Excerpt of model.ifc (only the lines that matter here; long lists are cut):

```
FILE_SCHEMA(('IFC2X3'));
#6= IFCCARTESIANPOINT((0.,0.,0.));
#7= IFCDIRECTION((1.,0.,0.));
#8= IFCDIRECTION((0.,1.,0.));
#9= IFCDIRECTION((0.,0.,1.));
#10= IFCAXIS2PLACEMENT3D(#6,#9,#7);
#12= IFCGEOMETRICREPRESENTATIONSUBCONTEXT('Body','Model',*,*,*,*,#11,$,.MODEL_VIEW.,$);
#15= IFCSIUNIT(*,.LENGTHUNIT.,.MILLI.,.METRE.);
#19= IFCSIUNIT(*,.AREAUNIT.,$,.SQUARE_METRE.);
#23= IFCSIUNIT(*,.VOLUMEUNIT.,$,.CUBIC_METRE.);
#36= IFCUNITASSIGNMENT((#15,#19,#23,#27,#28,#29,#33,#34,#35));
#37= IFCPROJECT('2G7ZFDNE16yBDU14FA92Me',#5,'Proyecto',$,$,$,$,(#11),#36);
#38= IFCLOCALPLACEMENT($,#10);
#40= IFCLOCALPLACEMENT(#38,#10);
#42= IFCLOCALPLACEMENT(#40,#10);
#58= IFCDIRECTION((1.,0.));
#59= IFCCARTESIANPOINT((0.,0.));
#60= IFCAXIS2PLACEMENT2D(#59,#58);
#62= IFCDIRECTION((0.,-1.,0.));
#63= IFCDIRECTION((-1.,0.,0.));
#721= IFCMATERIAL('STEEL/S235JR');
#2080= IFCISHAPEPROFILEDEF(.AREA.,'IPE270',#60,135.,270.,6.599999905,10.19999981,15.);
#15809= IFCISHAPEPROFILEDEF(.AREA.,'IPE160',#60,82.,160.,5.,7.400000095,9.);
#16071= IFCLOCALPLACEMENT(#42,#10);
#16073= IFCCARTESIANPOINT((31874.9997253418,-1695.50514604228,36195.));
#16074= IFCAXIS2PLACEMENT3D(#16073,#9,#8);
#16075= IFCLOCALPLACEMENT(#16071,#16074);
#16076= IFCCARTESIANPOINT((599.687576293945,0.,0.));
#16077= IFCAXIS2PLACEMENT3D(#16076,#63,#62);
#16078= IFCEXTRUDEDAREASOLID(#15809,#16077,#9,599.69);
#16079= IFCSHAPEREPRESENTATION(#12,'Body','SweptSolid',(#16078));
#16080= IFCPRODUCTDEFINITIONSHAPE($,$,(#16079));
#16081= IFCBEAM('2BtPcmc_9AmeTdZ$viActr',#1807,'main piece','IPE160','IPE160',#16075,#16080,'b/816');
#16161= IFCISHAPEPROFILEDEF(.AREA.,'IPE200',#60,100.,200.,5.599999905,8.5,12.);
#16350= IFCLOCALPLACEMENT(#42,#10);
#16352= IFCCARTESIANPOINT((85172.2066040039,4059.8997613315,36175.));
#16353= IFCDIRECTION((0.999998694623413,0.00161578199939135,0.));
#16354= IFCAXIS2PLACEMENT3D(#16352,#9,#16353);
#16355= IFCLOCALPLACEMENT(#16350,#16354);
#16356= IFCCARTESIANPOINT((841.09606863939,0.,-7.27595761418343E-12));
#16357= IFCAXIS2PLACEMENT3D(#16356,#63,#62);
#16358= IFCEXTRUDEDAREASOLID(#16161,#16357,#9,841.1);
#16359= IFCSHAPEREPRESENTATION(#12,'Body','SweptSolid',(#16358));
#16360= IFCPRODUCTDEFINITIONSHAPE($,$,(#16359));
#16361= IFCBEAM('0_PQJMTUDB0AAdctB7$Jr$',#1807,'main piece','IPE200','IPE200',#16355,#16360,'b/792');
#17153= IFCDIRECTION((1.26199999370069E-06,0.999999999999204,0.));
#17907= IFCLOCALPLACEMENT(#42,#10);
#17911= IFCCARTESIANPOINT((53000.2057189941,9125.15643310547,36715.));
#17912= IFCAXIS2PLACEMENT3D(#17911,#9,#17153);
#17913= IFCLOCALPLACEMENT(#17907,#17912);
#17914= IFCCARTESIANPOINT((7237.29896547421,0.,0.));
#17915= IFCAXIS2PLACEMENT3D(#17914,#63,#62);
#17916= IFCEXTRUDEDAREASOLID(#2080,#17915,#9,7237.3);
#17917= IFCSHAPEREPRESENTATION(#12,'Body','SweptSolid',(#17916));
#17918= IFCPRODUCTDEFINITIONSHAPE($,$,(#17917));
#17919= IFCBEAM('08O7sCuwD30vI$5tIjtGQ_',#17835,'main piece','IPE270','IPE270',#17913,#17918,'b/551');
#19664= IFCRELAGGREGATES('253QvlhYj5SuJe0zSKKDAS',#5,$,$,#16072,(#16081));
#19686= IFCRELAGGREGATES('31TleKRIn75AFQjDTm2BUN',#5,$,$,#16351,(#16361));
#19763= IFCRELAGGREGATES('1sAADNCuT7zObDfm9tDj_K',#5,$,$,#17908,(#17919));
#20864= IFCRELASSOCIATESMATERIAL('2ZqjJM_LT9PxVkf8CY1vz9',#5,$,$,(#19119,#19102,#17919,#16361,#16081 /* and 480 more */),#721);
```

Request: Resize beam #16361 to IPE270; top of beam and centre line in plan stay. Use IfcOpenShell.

```python
import ifcopenshell
import ifcopenshell.util.element
import ifcopenshell.util.representation

model = ifcopenshell.open("model.ifc")

member = model.by_guid("0_PQJMTUDB0AAdctB7$Jr$")
source = next(p for p in model.by_type("IfcIShapeProfileDef") if p.ProfileName == "IPE270")

body = ifcopenshell.util.representation.get_representation(member, "Model", "Body")
solid = body.Items[0]
old_profile = solid.SweptArea

# Copy the section's sizes but keep this member's own profile position.
profile = ifcopenshell.util.element.copy(model, source)
# Profiles are centred, so shift by half the change in depth to hold the top.
shift = (old_profile.OverallDepth - profile.OverallDepth) / 2
x, y = old_profile.Position.Location.Coordinates
up = (0.0, 1.0)  # upwards, in the solid's own plane
location = model.createIfcCartesianPoint((x + up[0] * shift, y + up[1] * shift))
profile.Position = model.createIfcAxis2Placement2D(location, old_profile.Position.RefDirection)
solid.SweptArea = profile
if not model.get_total_inverses(old_profile):
    ifcopenshell.util.element.remove_deep2(model, old_profile)
member.Description = member.Description.replace("IPE200", "IPE270")
member.ObjectType = member.ObjectType.replace("IPE200", "IPE270")

print(solid.SweptArea)

model.write("model_v2.ifc")
```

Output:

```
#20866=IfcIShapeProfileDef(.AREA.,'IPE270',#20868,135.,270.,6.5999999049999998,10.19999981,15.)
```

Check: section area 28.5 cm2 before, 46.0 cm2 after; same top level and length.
